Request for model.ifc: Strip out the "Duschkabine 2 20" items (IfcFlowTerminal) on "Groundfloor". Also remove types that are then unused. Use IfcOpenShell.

First a look at what the model holds.

```python
import ifcopenshell
import ifcopenshell.util.element

model = ifcopenshell.open("model.ifc")
print(model.schema)
storey = next(s for s in model.by_type("IfcBuildingStorey") if s.Name == "Groundfloor")
terminals = [e for e in ifcopenshell.util.element.get_decomposition(storey) if e.is_a("IfcFlowTerminal")]
seen = {}
for e in terminals:
    element_type = ifcopenshell.util.element.get_type(e)
    name = element_type.Name if element_type not in (None, e) else None
    seen[name] = seen.get(name, 0) + 1
for name, count in sorted(seen.items(), key=str):
    print(count, "x", name)
```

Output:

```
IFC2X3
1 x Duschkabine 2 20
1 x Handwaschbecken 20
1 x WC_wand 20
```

```python
import ifcopenshell
import ifcopenshell.api.root
import ifcopenshell.util.element

model = ifcopenshell.open("model.ifc")

storey = next(s for s in model.by_type("IfcBuildingStorey") if s.Name == "Groundfloor")
terminals = [e for e in ifcopenshell.util.element.get_decomposition(storey) if e.is_a("IfcFlowTerminal")]
targets = [e for e in terminals if (t := ifcopenshell.util.element.get_type(e)) not in (None, e) and t.Name == "Duschkabine 2 20"]
types = {ifcopenshell.util.element.get_type(e) for e in targets} - {None, *targets}

for e in targets:
    ifcopenshell.api.root.remove_product(model, product=e)
print(len(targets), "removed")

unused = [t for t in types if not ifcopenshell.util.element.get_types(t)]
for t in unused:
    ifcopenshell.api.root.remove_product(model, product=t)
print(len(unused), "unused types removed")

model.write("model_updated.ifc")
```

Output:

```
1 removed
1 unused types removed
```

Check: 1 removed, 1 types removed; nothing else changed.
